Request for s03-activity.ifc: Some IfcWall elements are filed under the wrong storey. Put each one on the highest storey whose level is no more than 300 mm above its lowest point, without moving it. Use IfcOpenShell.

First a look at what the model holds.

```python
import ifcopenshell
import ifcopenshell.util.element
import ifcopenshell.util.placement

model = ifcopenshell.open("s03-activity.ifc")
print(model.schema)
for storey in model.by_type("IfcBuildingStorey"):
    level = ifcopenshell.util.placement.get_storey_elevation(storey)
    count = sum(e.is_a("IfcWall") for e in ifcopenshell.util.element.get_contained(storey))
    print(storey.id(), storey.Name, round(level, 3), count, sep=" | ")
```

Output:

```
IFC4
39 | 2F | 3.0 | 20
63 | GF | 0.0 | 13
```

```python
import ifcopenshell
import ifcopenshell.api.spatial
import ifcopenshell.geom
import ifcopenshell.util.element
import ifcopenshell.util.placement
import ifcopenshell.util.shape
import ifcopenshell.util.unit

model = ifcopenshell.open("s03-activity.ifc")
unit_scale = ifcopenshell.util.unit.calculate_unit_scale(model)
settings = ifcopenshell.geom.settings()

levels = sorted(
    ((ifcopenshell.util.placement.get_storey_elevation(s) * unit_scale, s) for s in model.by_type("IfcBuildingStorey")),
    key=lambda pair: pair[0],
)

for e in model.by_type("IfcWall"):
    current = e.ContainedInStructure[0].RelatingStructure if e.ContainedInStructure else None
    if current is None or not current.is_a("IfcBuildingStorey"):
        continue
    shape = ifcopenshell.geom.create_shape(settings, e)
    bottom = ifcopenshell.util.shape.get_shape_bottom_elevation(shape, shape.geometry)
    below = [s for level, s in levels if level <= bottom + 0.3]
    storey = below[-1] if below else levels[0][1]
    if storey != current:
        # assign_container keeps the world position.
        ifcopenshell.api.spatial.assign_container(model, products=[e], relating_structure=storey)
        print(e.id(), current.Name, "->", storey.Name)

model.write("s03-activity_v2.ifc")
```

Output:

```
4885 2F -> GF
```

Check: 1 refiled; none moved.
